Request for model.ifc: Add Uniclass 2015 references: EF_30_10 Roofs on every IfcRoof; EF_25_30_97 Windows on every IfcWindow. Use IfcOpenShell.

First a look at what the model holds.

```python
import ifcopenshell

model = ifcopenshell.open("model.ifc")
print(model.schema)
print("classifications:", [c.Name for c in model.by_type("IfcClassification")])
for ifc_class in ("IfcDoor", "IfcRoof", "IfcStair", "IfcWall", "IfcWindow"):
    print(ifc_class, len(model.by_type(ifc_class)))
```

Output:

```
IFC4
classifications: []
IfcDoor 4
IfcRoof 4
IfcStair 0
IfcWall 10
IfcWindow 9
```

```python
import ifcopenshell
import ifcopenshell.api.classification

model = ifcopenshell.open("model.ifc")

system = ifcopenshell.api.classification.add_classification(model, classification="Uniclass 2015")

codes = {
    "IfcRoof": ("EF_30_10", "Roofs"),
    "IfcWindow": ("EF_25_30_97", "Windows"),
}
for ifc_class, (code, name) in codes.items():
    products = model.by_type(ifc_class)
    ifcopenshell.api.classification.add_reference(
        model, products=products, classification=system, identification=code, name=name
    )
    print(code, len(products))

model.write("model-out.ifc")
```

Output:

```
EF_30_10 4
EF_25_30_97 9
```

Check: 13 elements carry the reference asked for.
